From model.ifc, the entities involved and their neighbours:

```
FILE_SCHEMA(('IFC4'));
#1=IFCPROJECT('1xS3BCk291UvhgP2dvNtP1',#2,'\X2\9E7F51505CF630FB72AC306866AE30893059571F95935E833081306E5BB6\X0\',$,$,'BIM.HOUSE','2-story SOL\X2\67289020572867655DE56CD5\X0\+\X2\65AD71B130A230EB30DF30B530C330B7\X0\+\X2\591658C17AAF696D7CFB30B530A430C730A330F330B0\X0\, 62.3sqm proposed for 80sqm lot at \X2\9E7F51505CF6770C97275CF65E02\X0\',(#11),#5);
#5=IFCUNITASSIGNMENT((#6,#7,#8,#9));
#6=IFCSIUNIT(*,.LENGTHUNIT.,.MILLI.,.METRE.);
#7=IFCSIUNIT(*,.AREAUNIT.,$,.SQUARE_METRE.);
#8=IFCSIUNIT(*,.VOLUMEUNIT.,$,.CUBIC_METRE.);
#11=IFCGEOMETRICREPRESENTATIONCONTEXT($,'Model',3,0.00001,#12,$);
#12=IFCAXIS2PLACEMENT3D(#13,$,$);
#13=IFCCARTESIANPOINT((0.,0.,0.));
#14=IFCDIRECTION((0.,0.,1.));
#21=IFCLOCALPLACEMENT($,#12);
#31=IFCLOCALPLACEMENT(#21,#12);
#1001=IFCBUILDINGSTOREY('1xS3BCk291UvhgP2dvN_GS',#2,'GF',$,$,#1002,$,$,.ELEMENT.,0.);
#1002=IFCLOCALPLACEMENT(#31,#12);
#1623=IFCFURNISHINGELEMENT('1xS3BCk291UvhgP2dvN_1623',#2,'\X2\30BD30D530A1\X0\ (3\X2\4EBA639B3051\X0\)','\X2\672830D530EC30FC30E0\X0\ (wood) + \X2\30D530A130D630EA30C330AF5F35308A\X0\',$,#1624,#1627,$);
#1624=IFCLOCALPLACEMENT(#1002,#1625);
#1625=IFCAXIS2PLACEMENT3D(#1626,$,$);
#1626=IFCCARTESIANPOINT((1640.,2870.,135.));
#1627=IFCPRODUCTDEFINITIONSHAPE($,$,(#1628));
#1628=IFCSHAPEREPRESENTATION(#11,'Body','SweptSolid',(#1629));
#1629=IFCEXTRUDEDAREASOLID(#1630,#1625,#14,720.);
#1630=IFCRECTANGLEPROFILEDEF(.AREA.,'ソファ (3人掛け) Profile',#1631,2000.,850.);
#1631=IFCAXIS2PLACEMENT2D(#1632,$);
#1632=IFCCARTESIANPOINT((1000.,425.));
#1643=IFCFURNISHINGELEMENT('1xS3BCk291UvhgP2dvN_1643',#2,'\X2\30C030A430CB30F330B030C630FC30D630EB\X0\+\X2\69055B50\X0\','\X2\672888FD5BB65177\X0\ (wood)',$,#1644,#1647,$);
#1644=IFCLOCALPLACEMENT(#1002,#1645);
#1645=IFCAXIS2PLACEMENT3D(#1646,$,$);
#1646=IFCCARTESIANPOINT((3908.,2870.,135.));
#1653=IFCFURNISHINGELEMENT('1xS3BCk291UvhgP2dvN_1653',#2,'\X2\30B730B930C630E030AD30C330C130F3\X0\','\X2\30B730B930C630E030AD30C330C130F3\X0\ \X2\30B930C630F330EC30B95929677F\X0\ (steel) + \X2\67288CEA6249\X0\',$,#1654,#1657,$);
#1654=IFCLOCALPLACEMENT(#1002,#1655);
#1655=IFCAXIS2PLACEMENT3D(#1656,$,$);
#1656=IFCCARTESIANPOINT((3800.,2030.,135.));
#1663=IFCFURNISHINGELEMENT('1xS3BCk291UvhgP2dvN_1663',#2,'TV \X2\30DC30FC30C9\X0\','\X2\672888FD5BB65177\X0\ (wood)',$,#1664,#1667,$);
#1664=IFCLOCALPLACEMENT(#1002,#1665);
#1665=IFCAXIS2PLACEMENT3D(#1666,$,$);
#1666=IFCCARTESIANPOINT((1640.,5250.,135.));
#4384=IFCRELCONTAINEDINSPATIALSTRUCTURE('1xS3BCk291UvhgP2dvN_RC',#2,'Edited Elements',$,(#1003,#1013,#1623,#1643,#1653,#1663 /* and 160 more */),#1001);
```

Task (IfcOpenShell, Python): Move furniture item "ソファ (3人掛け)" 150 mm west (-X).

```python
import ifcopenshell
import ifcopenshell.api.geometry
import ifcopenshell.util.placement

model = ifcopenshell.open("model.ifc")

item = model.by_guid("1xS3BCk291UvhgP2dvN_1623")
matrix = ifcopenshell.util.placement.get_local_placement(item.ObjectPlacement)
matrix[0, 3] -= 150.0
ifcopenshell.api.geometry.edit_object_placement(model, product=item, matrix=matrix, is_si=False)

print(ifcopenshell.util.placement.get_local_placement(item.ObjectPlacement).round(3) + 0.0)

model.write("model_v2.ifc")
```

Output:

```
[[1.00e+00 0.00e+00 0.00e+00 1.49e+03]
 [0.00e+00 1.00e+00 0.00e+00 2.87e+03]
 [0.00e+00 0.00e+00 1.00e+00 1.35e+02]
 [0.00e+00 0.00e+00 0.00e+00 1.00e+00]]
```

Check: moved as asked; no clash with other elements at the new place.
